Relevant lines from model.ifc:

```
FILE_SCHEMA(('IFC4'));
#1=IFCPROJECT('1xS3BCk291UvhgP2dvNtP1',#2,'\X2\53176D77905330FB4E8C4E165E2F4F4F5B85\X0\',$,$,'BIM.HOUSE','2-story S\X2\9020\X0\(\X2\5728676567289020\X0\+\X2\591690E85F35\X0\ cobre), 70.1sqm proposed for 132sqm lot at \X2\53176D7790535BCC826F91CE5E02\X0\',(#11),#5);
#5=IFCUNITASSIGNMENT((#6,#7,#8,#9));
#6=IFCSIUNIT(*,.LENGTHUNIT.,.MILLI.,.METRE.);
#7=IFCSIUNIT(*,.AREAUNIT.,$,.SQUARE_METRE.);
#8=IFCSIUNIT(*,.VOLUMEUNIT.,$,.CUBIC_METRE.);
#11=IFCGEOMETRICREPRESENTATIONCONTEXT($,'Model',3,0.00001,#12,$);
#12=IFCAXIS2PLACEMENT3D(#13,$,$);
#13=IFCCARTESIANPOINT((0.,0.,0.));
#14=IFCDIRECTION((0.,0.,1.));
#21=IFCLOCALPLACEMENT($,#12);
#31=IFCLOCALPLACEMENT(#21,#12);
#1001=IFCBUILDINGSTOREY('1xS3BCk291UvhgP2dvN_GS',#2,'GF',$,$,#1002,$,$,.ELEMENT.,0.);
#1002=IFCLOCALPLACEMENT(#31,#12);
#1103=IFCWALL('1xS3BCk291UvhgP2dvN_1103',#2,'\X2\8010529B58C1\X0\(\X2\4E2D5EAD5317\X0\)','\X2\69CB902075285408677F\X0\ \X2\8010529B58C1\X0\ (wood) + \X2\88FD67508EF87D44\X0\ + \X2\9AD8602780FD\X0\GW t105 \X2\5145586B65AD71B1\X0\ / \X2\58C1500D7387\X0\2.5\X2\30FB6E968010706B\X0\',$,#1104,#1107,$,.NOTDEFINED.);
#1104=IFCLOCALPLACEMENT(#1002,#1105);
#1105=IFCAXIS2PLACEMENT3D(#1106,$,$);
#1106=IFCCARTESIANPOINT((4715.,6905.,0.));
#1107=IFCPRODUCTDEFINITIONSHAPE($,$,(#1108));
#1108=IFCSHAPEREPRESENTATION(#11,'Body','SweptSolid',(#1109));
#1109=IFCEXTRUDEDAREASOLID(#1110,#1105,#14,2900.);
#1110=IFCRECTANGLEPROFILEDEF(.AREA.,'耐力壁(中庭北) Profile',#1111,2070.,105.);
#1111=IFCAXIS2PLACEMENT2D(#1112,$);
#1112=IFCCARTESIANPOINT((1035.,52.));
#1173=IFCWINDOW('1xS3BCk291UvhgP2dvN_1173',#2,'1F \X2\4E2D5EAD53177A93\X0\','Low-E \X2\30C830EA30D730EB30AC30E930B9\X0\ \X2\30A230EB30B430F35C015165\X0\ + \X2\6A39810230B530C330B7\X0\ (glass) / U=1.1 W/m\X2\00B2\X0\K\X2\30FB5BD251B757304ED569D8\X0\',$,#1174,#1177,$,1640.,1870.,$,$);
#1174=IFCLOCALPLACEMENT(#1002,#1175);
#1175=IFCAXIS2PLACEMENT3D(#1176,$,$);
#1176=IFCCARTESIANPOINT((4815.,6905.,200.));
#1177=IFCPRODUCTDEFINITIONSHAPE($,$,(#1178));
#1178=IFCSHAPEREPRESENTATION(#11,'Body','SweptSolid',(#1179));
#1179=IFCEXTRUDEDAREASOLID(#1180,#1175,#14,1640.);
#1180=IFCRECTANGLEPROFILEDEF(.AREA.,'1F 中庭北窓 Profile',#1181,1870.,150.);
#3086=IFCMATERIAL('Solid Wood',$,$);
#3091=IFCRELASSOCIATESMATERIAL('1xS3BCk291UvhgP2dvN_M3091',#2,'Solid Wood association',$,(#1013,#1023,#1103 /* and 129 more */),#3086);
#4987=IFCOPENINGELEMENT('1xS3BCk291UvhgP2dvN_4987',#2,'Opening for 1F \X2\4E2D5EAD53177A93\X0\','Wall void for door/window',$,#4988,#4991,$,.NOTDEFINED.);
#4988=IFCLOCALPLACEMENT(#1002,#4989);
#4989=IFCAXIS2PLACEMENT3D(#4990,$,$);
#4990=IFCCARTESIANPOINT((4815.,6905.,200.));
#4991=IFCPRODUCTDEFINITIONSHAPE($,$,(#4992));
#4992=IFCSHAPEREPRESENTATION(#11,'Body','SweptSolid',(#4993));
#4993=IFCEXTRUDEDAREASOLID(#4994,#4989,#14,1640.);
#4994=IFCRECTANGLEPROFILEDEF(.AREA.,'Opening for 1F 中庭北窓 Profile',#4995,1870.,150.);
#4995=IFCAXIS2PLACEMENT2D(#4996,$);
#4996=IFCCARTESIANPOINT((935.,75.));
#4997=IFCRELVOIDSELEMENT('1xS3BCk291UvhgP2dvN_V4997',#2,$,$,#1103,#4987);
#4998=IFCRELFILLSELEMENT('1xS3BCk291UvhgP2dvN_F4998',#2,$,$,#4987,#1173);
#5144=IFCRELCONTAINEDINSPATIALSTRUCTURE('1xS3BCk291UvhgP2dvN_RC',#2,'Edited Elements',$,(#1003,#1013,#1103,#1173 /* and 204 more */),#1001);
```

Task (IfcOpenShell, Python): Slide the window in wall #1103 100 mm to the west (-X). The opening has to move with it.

```python
import ifcopenshell
import ifcopenshell.api.geometry
import ifcopenshell.util.placement
import ifcopenshell.util.unit

model = ifcopenshell.open("model.ifc")
unit_scale = ifcopenshell.util.unit.calculate_unit_scale(model)

window = model.by_id(1173)
opening = window.FillsVoids[0].RelatingOpeningElement
wall = opening.VoidsElements[0].RelatingBuildingElement

wall_matrix = ifcopenshell.util.placement.get_local_placement(wall.ObjectPlacement)
shift = wall_matrix[:3, 0] * -0.1 / unit_scale
before = ifcopenshell.util.placement.get_local_placement(window.ObjectPlacement)[:3, 3].copy()

# The window is not placed relative to its opening, so move both.
for product in (opening, window):
    matrix = ifcopenshell.util.placement.get_local_placement(product.ObjectPlacement)
    matrix[:3, 3] += shift
    ifcopenshell.api.geometry.edit_object_placement(model, product=product, matrix=matrix, is_si=False)

after = ifcopenshell.util.placement.get_local_placement(window.ObjectPlacement)[:3, 3]
print("window moved by", (after - before).round(3) + 0.0)

model.write("model_v2.ifc")
```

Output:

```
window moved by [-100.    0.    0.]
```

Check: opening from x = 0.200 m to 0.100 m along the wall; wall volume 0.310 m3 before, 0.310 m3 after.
